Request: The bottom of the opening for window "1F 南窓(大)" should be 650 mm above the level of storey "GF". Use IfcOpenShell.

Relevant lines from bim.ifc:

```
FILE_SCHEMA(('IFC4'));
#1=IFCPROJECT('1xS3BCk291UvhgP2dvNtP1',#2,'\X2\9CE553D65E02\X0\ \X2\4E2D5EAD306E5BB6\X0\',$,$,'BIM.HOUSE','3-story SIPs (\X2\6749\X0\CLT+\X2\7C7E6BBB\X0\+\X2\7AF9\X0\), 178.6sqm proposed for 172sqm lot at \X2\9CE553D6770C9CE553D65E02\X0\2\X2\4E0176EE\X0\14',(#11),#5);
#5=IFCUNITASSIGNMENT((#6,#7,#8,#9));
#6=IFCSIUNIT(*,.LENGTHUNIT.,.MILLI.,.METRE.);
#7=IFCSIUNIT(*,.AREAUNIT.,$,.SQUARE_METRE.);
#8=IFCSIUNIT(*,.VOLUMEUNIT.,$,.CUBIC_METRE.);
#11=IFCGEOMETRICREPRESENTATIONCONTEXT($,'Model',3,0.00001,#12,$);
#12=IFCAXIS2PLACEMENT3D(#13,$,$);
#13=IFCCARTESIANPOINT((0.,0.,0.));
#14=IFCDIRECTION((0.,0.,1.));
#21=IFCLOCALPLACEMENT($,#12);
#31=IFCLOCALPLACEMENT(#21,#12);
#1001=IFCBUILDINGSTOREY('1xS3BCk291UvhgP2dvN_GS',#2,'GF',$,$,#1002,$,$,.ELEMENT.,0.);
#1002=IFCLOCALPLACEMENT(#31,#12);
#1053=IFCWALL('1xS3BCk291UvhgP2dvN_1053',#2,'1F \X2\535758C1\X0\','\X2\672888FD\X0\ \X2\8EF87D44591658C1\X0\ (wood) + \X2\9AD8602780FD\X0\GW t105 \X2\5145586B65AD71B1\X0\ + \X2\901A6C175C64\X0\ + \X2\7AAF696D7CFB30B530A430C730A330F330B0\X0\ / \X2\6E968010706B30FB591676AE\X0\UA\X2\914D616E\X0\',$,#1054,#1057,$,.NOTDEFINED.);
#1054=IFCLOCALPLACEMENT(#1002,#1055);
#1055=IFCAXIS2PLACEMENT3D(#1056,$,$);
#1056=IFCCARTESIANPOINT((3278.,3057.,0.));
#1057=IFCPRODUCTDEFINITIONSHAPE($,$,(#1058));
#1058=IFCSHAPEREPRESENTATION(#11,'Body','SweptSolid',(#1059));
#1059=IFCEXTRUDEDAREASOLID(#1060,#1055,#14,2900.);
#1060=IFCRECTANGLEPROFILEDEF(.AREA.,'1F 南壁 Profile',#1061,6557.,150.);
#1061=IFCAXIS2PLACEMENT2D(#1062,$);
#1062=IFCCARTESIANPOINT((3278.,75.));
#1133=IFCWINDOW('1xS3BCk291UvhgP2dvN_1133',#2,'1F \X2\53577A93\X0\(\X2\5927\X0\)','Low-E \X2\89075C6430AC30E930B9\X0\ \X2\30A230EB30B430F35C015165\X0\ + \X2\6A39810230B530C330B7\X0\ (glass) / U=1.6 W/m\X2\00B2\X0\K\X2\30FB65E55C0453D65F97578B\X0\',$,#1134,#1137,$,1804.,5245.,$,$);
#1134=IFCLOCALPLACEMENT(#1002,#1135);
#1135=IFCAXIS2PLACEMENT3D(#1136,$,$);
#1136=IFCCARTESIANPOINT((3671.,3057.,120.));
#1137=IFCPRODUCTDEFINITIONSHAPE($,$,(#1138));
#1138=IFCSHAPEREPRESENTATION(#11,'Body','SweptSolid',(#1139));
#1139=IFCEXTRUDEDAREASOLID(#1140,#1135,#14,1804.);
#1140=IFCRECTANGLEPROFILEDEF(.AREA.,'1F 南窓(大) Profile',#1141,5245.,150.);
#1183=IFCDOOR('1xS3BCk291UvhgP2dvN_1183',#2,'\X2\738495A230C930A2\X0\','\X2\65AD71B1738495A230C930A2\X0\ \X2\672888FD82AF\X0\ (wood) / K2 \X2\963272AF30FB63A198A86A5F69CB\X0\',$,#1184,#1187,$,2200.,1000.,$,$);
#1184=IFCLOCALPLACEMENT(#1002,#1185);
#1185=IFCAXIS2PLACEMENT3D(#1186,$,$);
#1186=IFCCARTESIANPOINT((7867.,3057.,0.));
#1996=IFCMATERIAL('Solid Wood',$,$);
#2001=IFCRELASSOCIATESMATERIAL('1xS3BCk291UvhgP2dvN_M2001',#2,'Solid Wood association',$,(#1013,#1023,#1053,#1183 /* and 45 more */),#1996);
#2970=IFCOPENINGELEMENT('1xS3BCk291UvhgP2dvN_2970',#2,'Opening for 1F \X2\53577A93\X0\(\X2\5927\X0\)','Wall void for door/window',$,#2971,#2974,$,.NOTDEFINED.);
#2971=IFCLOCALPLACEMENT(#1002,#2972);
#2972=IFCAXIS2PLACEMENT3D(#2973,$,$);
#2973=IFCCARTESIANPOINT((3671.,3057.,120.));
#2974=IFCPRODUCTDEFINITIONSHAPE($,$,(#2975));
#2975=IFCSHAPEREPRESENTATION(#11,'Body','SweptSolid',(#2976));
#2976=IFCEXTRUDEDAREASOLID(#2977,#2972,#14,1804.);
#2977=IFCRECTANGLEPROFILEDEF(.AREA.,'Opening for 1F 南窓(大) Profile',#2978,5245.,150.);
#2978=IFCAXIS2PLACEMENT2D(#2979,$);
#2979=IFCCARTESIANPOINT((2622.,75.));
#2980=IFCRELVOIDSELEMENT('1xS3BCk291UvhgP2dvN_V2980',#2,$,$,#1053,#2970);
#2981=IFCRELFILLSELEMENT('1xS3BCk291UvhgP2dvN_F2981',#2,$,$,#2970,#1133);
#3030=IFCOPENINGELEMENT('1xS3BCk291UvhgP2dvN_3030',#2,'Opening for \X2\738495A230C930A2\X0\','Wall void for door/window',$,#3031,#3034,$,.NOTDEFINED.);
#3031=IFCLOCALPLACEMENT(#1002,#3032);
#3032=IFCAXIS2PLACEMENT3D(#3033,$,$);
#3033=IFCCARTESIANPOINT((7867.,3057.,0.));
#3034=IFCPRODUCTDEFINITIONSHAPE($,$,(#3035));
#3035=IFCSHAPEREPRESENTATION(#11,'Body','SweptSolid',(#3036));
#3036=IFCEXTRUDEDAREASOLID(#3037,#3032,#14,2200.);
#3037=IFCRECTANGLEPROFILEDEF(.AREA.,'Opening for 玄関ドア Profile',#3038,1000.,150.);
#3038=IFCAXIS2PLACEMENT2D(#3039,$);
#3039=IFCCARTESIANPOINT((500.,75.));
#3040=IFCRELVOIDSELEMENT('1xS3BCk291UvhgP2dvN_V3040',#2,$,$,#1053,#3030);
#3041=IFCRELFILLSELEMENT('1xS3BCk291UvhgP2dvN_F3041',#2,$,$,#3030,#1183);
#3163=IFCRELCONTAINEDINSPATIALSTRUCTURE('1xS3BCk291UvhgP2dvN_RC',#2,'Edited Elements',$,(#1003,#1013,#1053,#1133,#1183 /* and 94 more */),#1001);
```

```python
import numpy as np
import ifcopenshell
import ifcopenshell.api.geometry
import ifcopenshell.geom
import ifcopenshell.util.element
import ifcopenshell.util.placement
import ifcopenshell.util.shape
import ifcopenshell.util.unit

model = ifcopenshell.open("bim.ifc")
unit_scale = ifcopenshell.util.unit.calculate_unit_scale(model)

window = model.by_id(1133)
opening = window.FillsVoids[0].RelatingOpeningElement
storey = ifcopenshell.util.element.get_container(window, ifc_class="IfcBuildingStorey")
level = ifcopenshell.util.placement.get_local_placement(storey.ObjectPlacement)[2, 3]

# The opening's origin need not be at the sill, so measure its lowest point.
shape = ifcopenshell.geom.create_shape(ifcopenshell.geom.settings(), opening)
bottom = ifcopenshell.util.shape.get_shape_bottom_elevation(shape, shape.geometry) / unit_scale
dz = level + 0.65 / unit_scale - bottom

shift = np.array([0.0, 0.0, dz])
# The window is not placed relative to its opening, so move both.
for product in (opening, window):
    matrix = ifcopenshell.util.placement.get_local_placement(product.ObjectPlacement)
    matrix[:3, 3] += shift
    ifcopenshell.api.geometry.edit_object_placement(model, product=product, matrix=matrix, is_si=False)

print(f"moved by {dz * unit_scale:+.3f} m")

model.write("bim_v2.ifc")
```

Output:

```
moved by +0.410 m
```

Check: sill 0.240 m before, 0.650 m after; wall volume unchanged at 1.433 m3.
